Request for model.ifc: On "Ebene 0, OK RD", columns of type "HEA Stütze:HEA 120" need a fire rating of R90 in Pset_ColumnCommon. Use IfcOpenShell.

First a look at what the model holds.

```python
import ifcopenshell
import ifcopenshell.util.element

model = ifcopenshell.open("model.ifc")
print(model.schema)
storey = next(s for s in model.by_type("IfcBuildingStorey") if s.Name == "Ebene 0, OK RD")
columns = [e for e in ifcopenshell.util.element.get_decomposition(storey) if e.is_a("IfcColumn")]
seen = {}
for e in columns:
    element_type = ifcopenshell.util.element.get_type(e)
    key = (element_type.Name if element_type != e and element_type else None, ifcopenshell.util.element.get_pset(e, "Pset_ColumnCommon", "FireRating"))
    seen[key] = seen.get(key, 0) + 1
for (name, value), count in sorted(seen.items(), key=str):
    print(count, "x", name, "|", value)
```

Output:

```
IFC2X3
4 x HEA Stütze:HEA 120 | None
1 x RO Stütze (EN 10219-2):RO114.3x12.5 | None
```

```python
import ifcopenshell
import ifcopenshell.api.pset
import ifcopenshell.util.element

model = ifcopenshell.open("model.ifc")

storey = next(s for s in model.by_type("IfcBuildingStorey") if s.Name == "Ebene 0, OK RD")
columns = [e for e in ifcopenshell.util.element.get_decomposition(storey) if e.is_a("IfcColumn")]

count = 0
for e in columns:
    element_type = ifcopenshell.util.element.get_type(e)
    if element_type in (None, e) or element_type.Name != "HEA Stütze:HEA 120":
        continue
    # add_pset returns the element's existing set when there is one.
    pset = ifcopenshell.api.pset.add_pset(model, product=e, name="Pset_ColumnCommon")
    ifcopenshell.api.pset.edit_pset(model, pset=pset, properties={"FireRating": "R90"})
    count += 1

print(count, "columns updated")

model.write("model_updated.ifc")
```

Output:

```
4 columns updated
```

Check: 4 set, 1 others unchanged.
